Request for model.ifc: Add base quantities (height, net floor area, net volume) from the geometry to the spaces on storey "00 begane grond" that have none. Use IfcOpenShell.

First a look at what the model holds.

```python
import ifcopenshell
import ifcopenshell.util.element
import ifcopenshell.util.unit

model = ifcopenshell.open("model.ifc")
print(model.schema)
for unit_type in ("LENGTHUNIT", "AREAUNIT", "VOLUMEUNIT"):
    print(unit_type, ifcopenshell.util.unit.calculate_unit_scale(model, unit_type))
storey = next(s for s in model.by_type("IfcBuildingStorey") if s.Name == "00 begane grond")
spaces = [e for e in ifcopenshell.util.element.get_decomposition(storey) if e.is_a("IfcSpace")]
for e in sorted(spaces, key=lambda e: e.id()):
    print(e.id(), e.is_a(), e.Name, list(ifcopenshell.util.element.get_psets(e, qtos_only=True)), sep=" | ")
```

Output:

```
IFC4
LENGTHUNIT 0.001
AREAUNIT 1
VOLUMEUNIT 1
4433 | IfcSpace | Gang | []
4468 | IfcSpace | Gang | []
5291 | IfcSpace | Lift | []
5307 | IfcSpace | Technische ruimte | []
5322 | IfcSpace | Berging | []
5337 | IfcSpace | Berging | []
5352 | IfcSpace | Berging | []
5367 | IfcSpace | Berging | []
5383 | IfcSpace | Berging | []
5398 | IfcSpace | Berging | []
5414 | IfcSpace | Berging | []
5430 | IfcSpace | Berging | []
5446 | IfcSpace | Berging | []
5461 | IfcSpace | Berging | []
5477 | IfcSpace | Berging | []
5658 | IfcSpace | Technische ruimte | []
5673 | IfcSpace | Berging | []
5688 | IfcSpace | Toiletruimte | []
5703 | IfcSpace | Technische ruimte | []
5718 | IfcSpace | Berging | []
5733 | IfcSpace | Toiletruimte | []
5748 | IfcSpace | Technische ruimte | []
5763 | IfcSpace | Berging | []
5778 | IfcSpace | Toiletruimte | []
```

```python
import ifcopenshell
import ifcopenshell.api.pset
import ifcopenshell.geom
import ifcopenshell.util.element
import ifcopenshell.util.shape
import ifcopenshell.util.unit

model = ifcopenshell.open("model.ifc")
unit_scale = ifcopenshell.util.unit.calculate_unit_scale(model)
area_scale = ifcopenshell.util.unit.calculate_unit_scale(model, "AREAUNIT")
volume_scale = ifcopenshell.util.unit.calculate_unit_scale(model, "VOLUMEUNIT")
settings = ifcopenshell.geom.settings()

storey = next(s for s in model.by_type("IfcBuildingStorey") if s.Name == "00 begane grond")
spaces = [e for e in ifcopenshell.util.element.get_decomposition(storey) if e.is_a("IfcSpace")]

for e in sorted(spaces, key=lambda e: e.id()):
    if ifcopenshell.util.element.get_psets(e, qtos_only=True, should_inherit=False):
        continue
    # Geometry comes back in metres, in the element's own axes.
    shape = ifcopenshell.geom.create_shape(settings, e)
    values = {
        "Height": ifcopenshell.util.shape.get_z(shape.geometry) / unit_scale,
        "NetFloorArea": ifcopenshell.util.shape.get_footprint_area(shape.geometry) / area_scale,
        "NetVolume": ifcopenshell.util.shape.get_volume(shape.geometry) / volume_scale,
    }
    qto = ifcopenshell.api.pset.add_qto(model, product=e, name="Qto_SpaceBaseQuantities")
    ifcopenshell.api.pset.edit_qto(model, qto=qto, properties=values)
    print(e.id(), {k: round(v, 3) for k, v in values.items()})

model.write("model_rev.ifc")
```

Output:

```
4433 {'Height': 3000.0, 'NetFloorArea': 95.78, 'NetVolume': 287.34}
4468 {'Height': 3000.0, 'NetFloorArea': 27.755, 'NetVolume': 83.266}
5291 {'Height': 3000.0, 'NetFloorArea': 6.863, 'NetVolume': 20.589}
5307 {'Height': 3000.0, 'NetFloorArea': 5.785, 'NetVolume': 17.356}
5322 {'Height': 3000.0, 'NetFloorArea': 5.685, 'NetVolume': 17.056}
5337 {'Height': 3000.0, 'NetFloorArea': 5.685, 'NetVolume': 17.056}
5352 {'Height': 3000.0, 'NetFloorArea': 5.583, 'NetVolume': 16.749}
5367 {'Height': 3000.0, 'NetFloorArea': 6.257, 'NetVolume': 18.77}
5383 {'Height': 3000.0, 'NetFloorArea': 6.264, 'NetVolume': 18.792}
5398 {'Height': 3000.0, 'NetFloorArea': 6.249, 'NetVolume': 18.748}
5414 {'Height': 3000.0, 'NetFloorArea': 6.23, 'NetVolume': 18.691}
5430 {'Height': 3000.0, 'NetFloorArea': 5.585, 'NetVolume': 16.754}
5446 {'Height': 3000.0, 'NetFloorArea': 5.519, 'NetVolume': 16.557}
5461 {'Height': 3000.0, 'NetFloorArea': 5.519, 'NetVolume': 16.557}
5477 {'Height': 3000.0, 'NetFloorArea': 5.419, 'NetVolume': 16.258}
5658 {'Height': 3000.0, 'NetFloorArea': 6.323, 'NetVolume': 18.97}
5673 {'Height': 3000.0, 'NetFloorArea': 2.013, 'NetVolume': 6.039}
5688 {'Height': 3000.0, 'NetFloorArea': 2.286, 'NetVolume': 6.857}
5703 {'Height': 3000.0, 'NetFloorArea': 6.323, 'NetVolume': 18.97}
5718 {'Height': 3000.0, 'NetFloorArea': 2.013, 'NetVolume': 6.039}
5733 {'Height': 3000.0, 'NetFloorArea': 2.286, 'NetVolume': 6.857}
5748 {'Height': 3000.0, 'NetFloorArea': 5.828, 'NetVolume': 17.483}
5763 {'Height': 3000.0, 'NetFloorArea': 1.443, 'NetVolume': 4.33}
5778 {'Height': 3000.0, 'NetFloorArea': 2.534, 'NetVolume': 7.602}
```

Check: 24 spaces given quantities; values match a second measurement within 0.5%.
